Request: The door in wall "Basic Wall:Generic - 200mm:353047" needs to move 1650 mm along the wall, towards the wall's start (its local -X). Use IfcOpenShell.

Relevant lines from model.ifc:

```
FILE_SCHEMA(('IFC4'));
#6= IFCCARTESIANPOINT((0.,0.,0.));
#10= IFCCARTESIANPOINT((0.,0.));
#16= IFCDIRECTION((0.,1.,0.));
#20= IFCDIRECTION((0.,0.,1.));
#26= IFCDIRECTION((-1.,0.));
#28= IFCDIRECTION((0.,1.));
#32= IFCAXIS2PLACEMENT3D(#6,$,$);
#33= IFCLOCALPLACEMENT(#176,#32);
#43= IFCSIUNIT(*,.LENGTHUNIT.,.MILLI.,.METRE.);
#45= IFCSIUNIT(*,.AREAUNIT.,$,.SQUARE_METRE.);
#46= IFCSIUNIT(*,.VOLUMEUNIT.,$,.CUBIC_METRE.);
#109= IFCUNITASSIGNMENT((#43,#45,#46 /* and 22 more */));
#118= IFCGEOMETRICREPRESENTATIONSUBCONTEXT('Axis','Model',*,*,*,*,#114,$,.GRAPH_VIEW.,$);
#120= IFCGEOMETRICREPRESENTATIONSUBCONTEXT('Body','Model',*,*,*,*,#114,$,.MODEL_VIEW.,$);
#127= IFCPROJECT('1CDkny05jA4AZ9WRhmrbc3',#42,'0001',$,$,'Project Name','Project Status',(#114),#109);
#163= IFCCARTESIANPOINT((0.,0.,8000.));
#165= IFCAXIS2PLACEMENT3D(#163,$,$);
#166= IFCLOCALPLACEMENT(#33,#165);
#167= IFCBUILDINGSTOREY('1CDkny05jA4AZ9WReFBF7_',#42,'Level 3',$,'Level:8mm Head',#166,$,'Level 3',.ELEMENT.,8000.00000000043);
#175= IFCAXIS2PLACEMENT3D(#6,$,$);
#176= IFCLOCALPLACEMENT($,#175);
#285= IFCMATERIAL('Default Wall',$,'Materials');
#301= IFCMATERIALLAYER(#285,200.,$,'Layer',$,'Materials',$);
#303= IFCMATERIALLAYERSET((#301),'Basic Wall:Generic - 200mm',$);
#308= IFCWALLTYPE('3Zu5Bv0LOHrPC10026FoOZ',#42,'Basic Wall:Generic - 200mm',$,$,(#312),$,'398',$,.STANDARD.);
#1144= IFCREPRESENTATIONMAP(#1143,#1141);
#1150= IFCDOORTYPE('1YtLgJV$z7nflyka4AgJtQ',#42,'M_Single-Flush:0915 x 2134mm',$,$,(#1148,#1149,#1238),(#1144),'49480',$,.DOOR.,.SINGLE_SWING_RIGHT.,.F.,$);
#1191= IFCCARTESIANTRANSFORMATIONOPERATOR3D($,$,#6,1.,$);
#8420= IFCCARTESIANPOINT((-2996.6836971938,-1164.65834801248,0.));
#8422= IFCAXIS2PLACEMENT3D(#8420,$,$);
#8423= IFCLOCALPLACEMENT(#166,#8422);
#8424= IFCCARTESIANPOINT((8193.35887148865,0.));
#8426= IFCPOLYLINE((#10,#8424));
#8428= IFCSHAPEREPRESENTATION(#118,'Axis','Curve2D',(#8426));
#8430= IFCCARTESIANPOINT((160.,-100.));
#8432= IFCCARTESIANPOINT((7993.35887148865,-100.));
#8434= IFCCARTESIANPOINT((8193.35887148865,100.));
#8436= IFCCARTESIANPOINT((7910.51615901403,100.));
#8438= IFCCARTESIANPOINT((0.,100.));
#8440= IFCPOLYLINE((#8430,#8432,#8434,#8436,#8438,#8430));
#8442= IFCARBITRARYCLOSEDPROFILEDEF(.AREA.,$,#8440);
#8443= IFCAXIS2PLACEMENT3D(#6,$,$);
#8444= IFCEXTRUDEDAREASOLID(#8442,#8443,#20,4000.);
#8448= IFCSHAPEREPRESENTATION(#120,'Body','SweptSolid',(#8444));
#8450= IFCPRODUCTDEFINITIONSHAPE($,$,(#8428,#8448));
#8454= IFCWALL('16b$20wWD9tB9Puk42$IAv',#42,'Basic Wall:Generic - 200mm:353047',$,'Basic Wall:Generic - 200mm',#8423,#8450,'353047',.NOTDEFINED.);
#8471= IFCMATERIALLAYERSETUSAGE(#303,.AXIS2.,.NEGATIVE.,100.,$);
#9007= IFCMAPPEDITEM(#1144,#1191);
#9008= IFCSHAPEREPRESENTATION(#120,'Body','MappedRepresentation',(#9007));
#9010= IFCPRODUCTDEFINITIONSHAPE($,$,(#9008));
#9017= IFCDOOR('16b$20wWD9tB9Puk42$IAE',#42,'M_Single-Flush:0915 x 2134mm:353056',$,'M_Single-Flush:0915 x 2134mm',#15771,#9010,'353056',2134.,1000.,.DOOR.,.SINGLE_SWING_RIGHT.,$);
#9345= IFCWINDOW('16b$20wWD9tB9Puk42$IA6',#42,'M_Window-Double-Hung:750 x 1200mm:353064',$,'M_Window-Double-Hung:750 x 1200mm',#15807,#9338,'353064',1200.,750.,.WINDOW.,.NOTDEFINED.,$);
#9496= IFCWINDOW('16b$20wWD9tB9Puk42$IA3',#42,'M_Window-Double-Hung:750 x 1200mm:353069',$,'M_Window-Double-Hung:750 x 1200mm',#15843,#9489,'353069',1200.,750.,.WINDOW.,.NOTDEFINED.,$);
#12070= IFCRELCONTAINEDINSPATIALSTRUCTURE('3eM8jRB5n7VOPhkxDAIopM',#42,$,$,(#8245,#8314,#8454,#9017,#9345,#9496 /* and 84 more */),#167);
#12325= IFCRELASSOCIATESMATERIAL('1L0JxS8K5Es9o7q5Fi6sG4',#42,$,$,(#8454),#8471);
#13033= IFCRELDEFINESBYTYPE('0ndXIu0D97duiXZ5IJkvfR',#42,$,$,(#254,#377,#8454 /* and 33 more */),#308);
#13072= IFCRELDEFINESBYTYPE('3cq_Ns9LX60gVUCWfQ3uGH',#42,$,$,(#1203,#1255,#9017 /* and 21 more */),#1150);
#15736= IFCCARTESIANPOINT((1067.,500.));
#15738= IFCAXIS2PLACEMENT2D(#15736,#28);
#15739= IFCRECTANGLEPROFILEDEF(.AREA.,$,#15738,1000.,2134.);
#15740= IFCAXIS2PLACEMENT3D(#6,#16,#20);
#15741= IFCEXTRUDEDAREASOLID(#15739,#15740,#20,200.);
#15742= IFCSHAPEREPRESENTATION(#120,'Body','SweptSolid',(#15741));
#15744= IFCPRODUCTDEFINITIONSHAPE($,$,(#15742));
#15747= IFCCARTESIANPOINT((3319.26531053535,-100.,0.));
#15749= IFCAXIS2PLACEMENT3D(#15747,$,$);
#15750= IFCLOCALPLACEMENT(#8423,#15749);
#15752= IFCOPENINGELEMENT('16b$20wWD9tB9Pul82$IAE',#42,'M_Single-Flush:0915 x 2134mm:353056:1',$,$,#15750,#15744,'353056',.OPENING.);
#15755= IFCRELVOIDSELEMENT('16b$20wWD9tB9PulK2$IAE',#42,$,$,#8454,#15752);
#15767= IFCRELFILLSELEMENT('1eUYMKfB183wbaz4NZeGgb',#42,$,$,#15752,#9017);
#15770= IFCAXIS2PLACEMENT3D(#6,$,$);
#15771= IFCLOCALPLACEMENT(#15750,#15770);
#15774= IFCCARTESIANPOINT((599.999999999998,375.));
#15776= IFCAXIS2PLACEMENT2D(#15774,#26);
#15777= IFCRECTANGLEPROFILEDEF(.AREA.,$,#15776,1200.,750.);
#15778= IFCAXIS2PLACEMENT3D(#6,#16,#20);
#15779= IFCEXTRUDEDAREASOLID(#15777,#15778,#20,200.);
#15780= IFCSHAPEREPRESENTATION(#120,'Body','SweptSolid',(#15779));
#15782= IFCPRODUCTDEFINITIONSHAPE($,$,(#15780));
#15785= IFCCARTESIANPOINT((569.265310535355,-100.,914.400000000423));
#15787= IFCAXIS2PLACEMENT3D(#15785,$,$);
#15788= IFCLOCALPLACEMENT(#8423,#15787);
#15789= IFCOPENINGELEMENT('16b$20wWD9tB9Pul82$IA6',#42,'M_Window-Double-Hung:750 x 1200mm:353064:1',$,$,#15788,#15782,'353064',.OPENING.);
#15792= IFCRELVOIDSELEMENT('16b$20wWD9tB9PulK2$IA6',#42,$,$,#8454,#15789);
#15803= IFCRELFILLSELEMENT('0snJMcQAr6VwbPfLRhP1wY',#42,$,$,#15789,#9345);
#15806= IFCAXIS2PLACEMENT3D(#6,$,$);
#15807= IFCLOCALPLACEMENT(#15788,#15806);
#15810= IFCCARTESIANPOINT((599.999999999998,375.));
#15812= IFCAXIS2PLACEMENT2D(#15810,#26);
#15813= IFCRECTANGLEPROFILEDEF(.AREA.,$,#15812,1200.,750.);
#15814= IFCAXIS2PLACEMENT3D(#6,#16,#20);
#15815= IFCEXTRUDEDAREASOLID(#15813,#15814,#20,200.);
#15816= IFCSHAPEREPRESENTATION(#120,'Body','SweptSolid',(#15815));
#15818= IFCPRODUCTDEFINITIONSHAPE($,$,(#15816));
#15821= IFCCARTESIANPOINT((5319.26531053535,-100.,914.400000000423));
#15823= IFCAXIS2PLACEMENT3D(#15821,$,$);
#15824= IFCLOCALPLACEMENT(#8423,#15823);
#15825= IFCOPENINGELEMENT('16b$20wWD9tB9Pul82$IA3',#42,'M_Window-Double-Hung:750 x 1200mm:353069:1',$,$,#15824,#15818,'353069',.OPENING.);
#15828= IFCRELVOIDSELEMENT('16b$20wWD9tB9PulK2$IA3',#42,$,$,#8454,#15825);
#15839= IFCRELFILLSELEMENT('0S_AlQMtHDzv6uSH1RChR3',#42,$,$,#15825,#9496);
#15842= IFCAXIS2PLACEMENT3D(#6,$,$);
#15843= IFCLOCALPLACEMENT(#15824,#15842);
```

```python
import ifcopenshell
import ifcopenshell.api.geometry
import ifcopenshell.util.placement
import ifcopenshell.util.unit

model = ifcopenshell.open("model.ifc")
unit_scale = ifcopenshell.util.unit.calculate_unit_scale(model)

door = model.by_guid("16b$20wWD9tB9Puk42$IAE")
opening = door.FillsVoids[0].RelatingOpeningElement
wall = opening.VoidsElements[0].RelatingBuildingElement

wall_matrix = ifcopenshell.util.placement.get_local_placement(wall.ObjectPlacement)
shift = wall_matrix[:3, 0] * -1.65 / unit_scale
before = ifcopenshell.util.placement.get_local_placement(door.ObjectPlacement)[:3, 3].copy()

# The door is placed relative to its opening, so it follows when the opening moves.
matrix = ifcopenshell.util.placement.get_local_placement(opening.ObjectPlacement)
matrix[:3, 3] += shift
ifcopenshell.api.geometry.edit_object_placement(
    model, product=opening, matrix=matrix, is_si=False, should_transform_children=True
)

after = ifcopenshell.util.placement.get_local_placement(door.ObjectPlacement)[:3, 3]
print("door moved by", (after - before).round(3) + 0.0)

model.write("model_v2.ifc")
```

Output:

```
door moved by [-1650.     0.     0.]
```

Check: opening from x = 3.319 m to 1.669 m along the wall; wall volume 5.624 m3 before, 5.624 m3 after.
